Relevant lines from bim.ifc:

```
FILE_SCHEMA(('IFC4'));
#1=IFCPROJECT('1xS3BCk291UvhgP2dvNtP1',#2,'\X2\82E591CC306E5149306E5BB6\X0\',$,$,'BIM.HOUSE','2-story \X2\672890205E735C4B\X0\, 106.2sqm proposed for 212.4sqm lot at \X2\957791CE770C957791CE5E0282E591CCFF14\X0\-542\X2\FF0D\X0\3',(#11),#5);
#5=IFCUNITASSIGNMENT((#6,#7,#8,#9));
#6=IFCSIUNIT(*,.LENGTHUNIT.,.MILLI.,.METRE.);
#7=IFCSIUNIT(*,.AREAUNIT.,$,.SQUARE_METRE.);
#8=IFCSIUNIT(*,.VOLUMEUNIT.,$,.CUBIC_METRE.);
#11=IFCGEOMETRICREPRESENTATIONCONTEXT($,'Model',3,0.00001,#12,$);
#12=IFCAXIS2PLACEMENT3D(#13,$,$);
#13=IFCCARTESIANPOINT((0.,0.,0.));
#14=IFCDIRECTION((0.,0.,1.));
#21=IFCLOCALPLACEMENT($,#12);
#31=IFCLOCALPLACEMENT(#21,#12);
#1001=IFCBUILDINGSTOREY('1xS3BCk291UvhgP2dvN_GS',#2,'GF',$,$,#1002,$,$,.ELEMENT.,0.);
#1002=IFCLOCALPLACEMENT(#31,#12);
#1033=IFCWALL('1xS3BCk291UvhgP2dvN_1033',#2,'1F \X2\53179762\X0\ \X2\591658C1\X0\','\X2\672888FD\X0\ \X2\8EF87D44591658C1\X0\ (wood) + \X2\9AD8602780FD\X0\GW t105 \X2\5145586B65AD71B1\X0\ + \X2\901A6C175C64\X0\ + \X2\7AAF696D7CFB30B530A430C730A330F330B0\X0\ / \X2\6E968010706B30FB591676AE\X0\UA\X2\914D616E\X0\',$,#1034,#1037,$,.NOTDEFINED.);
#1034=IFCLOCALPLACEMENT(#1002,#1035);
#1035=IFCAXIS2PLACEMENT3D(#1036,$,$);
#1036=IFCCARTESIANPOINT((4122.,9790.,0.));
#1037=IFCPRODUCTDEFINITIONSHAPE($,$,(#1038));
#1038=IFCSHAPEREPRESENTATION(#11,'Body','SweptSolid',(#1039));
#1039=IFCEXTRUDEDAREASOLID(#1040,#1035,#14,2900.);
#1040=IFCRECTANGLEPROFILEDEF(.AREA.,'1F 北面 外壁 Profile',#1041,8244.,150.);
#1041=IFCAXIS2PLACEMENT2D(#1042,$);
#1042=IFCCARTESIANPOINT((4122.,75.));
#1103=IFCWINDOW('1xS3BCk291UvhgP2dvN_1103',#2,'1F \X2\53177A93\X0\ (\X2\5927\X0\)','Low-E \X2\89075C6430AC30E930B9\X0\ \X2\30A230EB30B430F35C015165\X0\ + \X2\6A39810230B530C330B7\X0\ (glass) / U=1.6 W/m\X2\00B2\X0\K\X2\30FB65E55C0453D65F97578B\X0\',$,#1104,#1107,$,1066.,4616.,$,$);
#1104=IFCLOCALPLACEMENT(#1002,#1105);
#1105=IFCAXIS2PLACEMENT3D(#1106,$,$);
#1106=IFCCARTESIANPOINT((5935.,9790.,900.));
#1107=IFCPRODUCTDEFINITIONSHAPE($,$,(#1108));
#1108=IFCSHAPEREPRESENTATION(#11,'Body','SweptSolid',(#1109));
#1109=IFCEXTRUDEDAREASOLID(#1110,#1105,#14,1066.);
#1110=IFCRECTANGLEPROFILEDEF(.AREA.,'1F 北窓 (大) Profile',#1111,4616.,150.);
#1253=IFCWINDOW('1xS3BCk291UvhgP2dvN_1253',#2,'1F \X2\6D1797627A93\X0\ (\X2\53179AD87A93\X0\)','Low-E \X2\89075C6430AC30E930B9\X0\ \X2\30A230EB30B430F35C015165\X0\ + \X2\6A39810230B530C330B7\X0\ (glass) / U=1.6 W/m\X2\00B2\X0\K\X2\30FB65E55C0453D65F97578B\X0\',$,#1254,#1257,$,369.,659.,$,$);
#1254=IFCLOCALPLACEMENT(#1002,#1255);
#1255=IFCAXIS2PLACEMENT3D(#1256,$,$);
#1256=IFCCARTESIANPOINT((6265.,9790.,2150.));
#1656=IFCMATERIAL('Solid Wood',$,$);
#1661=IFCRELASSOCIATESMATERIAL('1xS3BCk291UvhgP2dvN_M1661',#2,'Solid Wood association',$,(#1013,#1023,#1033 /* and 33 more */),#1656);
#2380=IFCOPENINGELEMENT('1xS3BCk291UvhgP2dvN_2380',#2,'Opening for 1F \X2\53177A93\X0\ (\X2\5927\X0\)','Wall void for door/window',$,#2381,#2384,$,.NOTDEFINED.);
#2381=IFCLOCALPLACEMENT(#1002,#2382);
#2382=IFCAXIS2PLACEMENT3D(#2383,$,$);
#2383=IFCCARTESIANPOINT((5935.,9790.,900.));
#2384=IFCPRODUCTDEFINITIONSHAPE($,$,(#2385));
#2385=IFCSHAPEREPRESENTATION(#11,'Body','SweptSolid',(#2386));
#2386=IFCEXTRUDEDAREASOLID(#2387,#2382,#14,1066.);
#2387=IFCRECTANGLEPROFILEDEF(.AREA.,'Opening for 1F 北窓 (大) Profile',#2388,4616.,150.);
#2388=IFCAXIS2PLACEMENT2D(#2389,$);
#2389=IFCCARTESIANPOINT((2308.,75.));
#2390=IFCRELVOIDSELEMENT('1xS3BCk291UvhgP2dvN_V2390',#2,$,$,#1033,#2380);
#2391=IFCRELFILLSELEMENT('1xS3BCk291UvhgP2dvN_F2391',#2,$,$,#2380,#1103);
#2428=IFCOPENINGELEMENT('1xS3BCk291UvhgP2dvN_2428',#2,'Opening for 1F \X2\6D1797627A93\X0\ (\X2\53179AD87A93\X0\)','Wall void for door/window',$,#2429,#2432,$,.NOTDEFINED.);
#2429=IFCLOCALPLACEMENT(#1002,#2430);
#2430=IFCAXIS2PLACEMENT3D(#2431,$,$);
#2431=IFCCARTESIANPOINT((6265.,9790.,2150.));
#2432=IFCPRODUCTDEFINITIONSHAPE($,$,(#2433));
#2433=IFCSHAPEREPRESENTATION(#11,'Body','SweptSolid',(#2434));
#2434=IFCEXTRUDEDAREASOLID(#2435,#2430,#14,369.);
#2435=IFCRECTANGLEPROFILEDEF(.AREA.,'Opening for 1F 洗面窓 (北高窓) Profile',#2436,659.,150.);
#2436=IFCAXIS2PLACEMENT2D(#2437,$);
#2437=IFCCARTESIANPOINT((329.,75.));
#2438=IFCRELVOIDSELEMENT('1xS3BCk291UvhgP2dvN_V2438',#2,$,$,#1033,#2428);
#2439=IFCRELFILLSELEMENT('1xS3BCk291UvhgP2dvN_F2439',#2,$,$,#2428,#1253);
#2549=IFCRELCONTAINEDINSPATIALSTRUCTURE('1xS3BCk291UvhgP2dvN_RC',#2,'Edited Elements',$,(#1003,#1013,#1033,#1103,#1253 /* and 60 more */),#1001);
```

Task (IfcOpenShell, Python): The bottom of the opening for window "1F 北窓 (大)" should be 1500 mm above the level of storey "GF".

```python
import numpy as np
import ifcopenshell
import ifcopenshell.api.geometry
import ifcopenshell.geom
import ifcopenshell.util.element
import ifcopenshell.util.placement
import ifcopenshell.util.shape
import ifcopenshell.util.unit

model = ifcopenshell.open("bim.ifc")
unit_scale = ifcopenshell.util.unit.calculate_unit_scale(model)

window = model.by_guid("1xS3BCk291UvhgP2dvN_1103")
opening = window.FillsVoids[0].RelatingOpeningElement
storey = ifcopenshell.util.element.get_container(window, ifc_class="IfcBuildingStorey")
level = ifcopenshell.util.placement.get_local_placement(storey.ObjectPlacement)[2, 3]

# The opening's origin need not be at the sill, so measure its lowest point.
shape = ifcopenshell.geom.create_shape(ifcopenshell.geom.settings(), opening)
bottom = ifcopenshell.util.shape.get_shape_bottom_elevation(shape, shape.geometry) / unit_scale
dz = level + 1500.0 - bottom

shift = np.array([0.0, 0.0, dz])
# The window is not placed relative to its opening, so move both.
for product in (opening, window):
    matrix = ifcopenshell.util.placement.get_local_placement(product.ObjectPlacement)
    matrix[:3, 3] += shift
    ifcopenshell.api.geometry.edit_object_placement(model, product=product, matrix=matrix, is_si=False)

print(f"moved by {dz * unit_scale:+.3f} m")

model.write("bim_v2.ifc")
```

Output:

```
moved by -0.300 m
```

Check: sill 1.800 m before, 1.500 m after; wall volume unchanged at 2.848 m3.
